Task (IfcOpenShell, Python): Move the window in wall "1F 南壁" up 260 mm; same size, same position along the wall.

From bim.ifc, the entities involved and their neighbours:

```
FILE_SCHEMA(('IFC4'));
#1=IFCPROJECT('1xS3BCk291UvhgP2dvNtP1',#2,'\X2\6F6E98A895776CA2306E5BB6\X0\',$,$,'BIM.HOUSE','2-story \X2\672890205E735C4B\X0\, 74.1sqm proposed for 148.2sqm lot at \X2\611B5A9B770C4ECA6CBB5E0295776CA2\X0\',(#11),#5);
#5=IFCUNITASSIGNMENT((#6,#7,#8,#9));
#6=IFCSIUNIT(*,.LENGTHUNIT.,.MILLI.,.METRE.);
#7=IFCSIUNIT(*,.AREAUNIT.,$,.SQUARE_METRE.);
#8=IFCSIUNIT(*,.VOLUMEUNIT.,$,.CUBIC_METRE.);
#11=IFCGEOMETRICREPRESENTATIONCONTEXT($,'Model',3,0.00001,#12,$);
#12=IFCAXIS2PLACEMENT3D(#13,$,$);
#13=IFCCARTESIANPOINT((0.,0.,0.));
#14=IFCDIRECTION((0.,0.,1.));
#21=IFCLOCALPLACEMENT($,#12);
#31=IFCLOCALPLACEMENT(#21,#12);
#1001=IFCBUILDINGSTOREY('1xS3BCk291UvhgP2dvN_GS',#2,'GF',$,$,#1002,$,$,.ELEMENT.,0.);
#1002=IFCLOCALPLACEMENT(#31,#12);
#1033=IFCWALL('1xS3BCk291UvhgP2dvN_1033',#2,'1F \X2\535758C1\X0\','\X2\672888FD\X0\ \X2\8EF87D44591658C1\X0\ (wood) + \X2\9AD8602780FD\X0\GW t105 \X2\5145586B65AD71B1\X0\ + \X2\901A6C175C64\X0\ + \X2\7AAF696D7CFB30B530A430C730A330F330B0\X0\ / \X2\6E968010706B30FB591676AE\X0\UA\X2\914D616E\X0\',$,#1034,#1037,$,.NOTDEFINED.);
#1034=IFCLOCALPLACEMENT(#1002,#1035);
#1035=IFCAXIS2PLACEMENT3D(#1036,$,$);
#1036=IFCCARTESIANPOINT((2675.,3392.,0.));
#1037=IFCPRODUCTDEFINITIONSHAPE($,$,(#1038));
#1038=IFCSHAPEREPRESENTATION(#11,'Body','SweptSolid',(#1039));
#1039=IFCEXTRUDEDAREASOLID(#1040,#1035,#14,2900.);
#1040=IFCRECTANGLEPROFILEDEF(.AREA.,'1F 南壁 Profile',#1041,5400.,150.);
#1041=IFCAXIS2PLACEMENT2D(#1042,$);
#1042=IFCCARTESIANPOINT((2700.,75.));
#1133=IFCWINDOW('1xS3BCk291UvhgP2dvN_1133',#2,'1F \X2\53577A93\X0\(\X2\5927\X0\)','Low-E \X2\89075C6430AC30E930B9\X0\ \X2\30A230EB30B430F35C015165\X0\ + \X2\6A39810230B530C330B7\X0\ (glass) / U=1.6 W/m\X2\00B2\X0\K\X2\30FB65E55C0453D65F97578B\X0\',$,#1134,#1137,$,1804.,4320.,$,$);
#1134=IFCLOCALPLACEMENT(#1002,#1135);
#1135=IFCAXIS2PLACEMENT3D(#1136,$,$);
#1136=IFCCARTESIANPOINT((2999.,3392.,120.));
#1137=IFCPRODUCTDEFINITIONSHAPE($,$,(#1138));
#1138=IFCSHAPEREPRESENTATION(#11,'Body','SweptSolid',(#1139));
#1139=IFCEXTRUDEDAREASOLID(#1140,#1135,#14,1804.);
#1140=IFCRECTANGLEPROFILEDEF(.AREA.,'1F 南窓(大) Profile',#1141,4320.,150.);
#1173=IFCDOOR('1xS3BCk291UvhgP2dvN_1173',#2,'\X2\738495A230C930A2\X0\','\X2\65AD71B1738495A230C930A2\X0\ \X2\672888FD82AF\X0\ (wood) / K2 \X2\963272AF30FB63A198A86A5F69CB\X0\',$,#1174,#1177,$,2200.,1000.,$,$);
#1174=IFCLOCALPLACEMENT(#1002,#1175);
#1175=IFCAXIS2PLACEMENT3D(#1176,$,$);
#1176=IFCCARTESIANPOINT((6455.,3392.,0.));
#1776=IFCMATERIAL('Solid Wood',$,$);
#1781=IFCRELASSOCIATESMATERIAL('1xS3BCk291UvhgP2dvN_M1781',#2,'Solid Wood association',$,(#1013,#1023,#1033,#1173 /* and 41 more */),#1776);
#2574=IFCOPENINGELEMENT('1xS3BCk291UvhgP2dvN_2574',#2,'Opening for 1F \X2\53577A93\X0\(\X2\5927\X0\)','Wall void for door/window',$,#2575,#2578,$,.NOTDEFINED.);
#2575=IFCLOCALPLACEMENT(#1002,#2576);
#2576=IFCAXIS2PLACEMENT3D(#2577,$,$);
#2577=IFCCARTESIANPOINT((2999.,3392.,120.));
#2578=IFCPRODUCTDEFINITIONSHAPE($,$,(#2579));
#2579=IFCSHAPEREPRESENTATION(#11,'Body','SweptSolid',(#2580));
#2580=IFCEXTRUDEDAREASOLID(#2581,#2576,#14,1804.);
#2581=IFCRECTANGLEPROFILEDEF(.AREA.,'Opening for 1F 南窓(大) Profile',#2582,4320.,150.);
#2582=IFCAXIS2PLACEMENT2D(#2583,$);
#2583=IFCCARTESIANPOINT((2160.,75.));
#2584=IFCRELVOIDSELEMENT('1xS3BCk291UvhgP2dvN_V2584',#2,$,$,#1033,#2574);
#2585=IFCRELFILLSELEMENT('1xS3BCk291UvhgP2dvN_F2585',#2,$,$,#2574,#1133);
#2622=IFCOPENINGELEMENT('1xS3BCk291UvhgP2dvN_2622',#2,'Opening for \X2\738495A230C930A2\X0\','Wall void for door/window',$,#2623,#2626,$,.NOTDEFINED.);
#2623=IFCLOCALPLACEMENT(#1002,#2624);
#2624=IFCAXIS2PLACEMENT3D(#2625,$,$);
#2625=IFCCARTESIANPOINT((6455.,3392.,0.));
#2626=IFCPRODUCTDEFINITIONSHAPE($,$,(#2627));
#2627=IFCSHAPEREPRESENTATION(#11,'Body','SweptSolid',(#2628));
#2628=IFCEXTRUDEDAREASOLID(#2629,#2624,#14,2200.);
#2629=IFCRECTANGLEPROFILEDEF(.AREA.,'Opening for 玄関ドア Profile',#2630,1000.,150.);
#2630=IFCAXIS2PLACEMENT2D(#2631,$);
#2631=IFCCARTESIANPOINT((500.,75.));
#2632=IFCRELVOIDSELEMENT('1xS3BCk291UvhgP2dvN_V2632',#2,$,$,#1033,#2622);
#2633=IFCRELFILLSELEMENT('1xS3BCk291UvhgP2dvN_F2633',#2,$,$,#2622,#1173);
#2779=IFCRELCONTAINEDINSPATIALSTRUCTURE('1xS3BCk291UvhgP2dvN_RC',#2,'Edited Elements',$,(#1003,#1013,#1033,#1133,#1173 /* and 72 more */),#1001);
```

```python
import numpy as np
import ifcopenshell
import ifcopenshell.api.geometry
import ifcopenshell.util.placement
import ifcopenshell.util.unit

model = ifcopenshell.open("bim.ifc")
unit_scale = ifcopenshell.util.unit.calculate_unit_scale(model)

window = model.by_guid("1xS3BCk291UvhgP2dvN_1133")
opening = window.FillsVoids[0].RelatingOpeningElement
dz = 260.0

shift = np.array([0.0, 0.0, dz])
# The window is not placed relative to its opening, so move both.
for product in (opening, window):
    matrix = ifcopenshell.util.placement.get_local_placement(product.ObjectPlacement)
    matrix[:3, 3] += shift
    ifcopenshell.api.geometry.edit_object_placement(model, product=product, matrix=matrix, is_si=False)

print(f"moved by {dz * unit_scale:+.3f} m")

model.write("bim_rev.ifc")
```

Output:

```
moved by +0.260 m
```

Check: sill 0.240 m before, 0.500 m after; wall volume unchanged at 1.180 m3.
